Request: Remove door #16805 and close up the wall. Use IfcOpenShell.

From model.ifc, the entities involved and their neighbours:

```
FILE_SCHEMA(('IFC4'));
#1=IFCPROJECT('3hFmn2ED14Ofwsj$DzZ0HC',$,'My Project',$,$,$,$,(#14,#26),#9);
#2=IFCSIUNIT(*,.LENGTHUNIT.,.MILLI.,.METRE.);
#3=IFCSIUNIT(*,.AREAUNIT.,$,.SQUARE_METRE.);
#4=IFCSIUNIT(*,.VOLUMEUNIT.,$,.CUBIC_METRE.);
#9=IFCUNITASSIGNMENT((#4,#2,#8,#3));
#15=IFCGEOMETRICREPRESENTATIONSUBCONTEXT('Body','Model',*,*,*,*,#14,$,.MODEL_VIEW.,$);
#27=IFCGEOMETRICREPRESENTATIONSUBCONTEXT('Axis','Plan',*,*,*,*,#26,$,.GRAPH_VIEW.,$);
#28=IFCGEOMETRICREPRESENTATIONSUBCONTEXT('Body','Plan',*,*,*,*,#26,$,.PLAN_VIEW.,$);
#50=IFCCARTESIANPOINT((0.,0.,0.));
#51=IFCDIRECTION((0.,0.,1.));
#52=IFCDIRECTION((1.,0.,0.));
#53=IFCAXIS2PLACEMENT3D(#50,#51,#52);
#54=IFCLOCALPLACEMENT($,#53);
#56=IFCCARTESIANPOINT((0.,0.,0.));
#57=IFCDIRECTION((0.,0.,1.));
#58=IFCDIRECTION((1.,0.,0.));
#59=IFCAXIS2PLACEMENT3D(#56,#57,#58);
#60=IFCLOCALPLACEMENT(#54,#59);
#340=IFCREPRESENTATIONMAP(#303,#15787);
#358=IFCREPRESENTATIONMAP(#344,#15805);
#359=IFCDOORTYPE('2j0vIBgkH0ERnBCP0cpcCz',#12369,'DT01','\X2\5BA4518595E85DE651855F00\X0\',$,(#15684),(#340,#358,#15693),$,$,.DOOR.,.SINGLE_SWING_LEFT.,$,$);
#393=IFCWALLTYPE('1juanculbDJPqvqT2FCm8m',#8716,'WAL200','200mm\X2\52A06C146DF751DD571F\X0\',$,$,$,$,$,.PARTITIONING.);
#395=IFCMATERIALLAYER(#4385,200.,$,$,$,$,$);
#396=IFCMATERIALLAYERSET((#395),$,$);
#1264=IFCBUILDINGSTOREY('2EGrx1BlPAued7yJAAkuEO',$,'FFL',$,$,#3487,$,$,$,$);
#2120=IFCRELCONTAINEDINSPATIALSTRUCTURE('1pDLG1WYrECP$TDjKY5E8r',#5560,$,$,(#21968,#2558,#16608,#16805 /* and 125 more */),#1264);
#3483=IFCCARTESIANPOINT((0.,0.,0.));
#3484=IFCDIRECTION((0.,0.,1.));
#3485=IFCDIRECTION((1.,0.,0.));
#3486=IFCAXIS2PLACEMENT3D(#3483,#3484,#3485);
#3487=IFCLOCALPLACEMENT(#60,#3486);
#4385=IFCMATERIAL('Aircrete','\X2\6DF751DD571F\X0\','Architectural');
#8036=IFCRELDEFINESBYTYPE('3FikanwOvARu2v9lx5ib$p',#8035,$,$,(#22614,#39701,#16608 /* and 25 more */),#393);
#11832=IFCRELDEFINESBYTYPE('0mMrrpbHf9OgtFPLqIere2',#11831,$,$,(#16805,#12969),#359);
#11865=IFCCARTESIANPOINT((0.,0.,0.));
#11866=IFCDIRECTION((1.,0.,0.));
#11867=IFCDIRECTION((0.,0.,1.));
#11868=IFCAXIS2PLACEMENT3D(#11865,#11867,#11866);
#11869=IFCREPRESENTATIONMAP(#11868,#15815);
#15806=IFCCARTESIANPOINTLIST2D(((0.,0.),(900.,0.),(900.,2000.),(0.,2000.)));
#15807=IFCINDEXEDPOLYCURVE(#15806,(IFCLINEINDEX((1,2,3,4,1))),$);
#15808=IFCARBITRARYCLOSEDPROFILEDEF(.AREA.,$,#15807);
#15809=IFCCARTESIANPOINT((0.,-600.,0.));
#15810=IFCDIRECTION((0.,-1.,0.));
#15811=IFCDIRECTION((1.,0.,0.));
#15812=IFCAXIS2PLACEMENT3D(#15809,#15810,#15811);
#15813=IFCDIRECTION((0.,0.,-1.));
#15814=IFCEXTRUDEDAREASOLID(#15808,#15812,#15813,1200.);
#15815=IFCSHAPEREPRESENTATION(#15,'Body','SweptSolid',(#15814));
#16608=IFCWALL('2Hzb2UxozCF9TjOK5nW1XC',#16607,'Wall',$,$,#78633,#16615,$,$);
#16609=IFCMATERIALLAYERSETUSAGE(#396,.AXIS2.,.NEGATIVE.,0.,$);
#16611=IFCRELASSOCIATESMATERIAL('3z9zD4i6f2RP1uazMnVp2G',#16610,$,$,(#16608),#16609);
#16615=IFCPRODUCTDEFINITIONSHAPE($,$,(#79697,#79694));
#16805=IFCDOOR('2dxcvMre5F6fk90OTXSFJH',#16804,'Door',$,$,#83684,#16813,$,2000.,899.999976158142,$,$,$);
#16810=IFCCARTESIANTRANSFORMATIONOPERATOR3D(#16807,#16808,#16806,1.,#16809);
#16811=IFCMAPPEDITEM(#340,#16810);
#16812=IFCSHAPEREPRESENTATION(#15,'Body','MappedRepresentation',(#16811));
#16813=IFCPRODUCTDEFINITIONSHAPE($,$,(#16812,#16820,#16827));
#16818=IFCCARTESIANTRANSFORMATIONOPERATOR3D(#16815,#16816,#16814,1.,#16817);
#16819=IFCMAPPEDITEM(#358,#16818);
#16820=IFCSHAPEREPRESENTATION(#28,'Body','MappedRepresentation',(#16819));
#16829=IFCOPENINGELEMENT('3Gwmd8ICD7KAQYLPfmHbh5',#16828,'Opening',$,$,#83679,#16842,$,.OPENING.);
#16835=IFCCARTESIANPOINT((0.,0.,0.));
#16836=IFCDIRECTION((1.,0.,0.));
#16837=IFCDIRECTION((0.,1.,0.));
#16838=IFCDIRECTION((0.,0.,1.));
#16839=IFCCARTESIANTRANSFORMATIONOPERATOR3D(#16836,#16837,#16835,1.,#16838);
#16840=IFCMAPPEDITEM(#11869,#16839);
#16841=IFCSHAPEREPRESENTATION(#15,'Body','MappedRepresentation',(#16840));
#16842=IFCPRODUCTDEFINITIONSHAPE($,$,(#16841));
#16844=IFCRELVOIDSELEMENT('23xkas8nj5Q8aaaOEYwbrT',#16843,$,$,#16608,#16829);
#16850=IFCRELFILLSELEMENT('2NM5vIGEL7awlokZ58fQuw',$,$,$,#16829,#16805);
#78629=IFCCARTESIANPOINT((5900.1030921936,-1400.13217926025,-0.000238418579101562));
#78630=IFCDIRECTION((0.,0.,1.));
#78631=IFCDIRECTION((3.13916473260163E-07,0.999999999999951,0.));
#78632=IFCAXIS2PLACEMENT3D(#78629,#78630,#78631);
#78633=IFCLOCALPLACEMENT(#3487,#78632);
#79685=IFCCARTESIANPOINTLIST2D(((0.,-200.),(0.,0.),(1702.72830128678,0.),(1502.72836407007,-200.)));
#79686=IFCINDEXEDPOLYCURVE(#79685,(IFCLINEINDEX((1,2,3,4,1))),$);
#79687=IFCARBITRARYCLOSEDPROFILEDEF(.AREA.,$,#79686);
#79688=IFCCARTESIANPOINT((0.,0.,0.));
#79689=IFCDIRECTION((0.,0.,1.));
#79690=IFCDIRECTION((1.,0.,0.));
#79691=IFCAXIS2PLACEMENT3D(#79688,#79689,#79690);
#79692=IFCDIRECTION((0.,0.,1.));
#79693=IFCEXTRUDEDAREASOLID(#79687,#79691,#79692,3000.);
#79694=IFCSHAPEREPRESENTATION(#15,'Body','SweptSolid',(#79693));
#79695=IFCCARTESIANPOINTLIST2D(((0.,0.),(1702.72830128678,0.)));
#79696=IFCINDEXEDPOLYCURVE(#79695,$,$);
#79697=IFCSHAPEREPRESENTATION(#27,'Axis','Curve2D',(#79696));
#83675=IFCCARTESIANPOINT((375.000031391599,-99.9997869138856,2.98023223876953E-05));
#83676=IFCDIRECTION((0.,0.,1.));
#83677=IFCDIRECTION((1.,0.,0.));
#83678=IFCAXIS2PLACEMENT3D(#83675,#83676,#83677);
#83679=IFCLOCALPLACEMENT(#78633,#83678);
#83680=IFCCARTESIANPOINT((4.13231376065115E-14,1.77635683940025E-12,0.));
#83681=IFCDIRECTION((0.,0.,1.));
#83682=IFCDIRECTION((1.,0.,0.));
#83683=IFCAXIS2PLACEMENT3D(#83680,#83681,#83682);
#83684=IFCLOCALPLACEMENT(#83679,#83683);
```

```python
import ifcopenshell
import ifcopenshell.api.feature
import ifcopenshell.api.root
import ifcopenshell.geom
import ifcopenshell.util.shape

model = ifcopenshell.open("model.ifc")
settings = ifcopenshell.geom.settings()


def volume(element):
    """Net volume in cubic metres, openings subtracted."""
    shape = ifcopenshell.geom.create_shape(settings, element)
    return ifcopenshell.util.shape.get_volume(shape.geometry)


door = model.by_id(16805)
opening = door.FillsVoids[0].RelatingOpeningElement
wall = opening.VoidsElements[0].RelatingBuildingElement
before = volume(wall)

ifcopenshell.api.root.remove_product(model, product=door)
ifcopenshell.api.feature.remove_feature(model, feature=opening)

after = volume(wall)

print(f"wall volume {before:.3f} -> {after:.3f} m3")

model.write("model_edited.ifc")
```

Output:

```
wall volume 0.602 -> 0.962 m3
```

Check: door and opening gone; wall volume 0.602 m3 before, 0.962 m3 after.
